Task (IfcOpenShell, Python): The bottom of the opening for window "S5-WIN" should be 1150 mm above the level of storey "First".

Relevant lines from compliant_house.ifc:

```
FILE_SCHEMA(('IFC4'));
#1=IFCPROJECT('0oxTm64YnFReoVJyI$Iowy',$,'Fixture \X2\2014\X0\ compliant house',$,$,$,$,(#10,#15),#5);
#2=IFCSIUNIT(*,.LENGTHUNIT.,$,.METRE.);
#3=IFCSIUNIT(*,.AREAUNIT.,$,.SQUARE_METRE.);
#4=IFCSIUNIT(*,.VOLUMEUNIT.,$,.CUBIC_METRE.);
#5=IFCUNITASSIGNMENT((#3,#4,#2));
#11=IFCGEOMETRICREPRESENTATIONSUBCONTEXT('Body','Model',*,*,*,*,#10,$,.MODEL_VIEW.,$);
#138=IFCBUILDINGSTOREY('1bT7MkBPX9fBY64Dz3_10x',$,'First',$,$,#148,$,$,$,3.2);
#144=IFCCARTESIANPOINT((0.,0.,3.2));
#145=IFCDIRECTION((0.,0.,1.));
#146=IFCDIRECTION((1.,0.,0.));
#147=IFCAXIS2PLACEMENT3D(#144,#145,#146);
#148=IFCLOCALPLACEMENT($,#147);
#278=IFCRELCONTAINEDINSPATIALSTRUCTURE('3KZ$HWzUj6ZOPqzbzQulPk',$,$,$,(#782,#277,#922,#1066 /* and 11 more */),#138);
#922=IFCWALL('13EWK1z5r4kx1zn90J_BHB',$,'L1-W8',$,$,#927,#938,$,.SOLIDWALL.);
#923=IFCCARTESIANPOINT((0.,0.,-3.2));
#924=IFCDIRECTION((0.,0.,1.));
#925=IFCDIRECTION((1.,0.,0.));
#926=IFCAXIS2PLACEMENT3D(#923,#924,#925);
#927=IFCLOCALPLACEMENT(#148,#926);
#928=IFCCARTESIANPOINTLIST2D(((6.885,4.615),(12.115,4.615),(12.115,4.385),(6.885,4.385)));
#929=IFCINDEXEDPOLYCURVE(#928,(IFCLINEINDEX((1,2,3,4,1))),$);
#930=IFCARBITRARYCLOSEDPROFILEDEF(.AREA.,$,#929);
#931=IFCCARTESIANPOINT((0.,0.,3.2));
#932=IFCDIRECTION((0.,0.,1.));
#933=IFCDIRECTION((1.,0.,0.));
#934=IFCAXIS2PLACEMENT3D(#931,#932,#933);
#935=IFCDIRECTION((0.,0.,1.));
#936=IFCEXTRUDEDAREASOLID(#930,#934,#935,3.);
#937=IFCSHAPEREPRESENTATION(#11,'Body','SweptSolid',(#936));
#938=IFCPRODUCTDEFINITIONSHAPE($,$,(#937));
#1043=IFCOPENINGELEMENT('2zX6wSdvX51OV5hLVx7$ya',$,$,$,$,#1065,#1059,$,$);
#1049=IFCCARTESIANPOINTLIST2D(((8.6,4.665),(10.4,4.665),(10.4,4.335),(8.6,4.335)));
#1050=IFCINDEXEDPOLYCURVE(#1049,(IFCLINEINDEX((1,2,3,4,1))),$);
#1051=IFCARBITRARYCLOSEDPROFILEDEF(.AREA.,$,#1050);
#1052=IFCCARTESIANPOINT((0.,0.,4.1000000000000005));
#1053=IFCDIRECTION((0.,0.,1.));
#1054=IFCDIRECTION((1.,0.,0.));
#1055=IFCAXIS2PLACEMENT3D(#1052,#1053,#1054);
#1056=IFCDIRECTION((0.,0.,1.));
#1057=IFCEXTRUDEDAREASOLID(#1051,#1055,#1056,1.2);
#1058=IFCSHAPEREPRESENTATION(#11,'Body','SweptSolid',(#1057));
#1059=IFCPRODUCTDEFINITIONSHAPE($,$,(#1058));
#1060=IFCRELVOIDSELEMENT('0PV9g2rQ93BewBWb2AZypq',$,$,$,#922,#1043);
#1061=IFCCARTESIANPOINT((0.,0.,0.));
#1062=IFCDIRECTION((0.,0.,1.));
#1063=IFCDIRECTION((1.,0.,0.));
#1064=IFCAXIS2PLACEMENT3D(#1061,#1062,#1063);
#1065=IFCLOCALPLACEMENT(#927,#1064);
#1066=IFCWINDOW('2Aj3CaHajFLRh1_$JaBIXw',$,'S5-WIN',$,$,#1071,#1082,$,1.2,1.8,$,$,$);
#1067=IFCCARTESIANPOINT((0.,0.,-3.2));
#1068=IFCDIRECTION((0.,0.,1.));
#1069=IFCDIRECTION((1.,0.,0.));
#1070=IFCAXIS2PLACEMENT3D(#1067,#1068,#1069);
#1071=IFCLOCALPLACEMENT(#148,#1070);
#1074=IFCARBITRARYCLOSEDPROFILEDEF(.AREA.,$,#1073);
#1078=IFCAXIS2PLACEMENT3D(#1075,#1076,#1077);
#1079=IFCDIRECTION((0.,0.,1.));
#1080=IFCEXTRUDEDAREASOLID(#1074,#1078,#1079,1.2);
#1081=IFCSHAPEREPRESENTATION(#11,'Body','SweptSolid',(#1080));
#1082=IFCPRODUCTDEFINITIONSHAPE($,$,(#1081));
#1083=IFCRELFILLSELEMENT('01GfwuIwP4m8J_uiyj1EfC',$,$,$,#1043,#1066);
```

```python
import numpy as np
import ifcopenshell
import ifcopenshell.api.geometry
import ifcopenshell.geom
import ifcopenshell.util.element
import ifcopenshell.util.placement
import ifcopenshell.util.shape
import ifcopenshell.util.unit

model = ifcopenshell.open("compliant_house.ifc")
unit_scale = ifcopenshell.util.unit.calculate_unit_scale(model)

window = model.by_guid("2Aj3CaHajFLRh1_$JaBIXw")
opening = window.FillsVoids[0].RelatingOpeningElement
storey = ifcopenshell.util.element.get_container(window, ifc_class="IfcBuildingStorey")
level = ifcopenshell.util.placement.get_local_placement(storey.ObjectPlacement)[2, 3]

# The opening's origin need not be at the sill, so measure its lowest point.
shape = ifcopenshell.geom.create_shape(ifcopenshell.geom.settings(), opening)
bottom = ifcopenshell.util.shape.get_shape_bottom_elevation(shape, shape.geometry) / unit_scale
dz = level + 1.15 / unit_scale - bottom

shift = np.array([0.0, 0.0, dz])
# The window is not placed relative to its opening, so move both.
for product in (opening, window):
    matrix = ifcopenshell.util.placement.get_local_placement(product.ObjectPlacement)
    matrix[:3, 3] += shift
    ifcopenshell.api.geometry.edit_object_placement(model, product=product, matrix=matrix, is_si=False)

print(f"moved by {dz * unit_scale:+.3f} m")

model.write("compliant_house_edited.ifc")
```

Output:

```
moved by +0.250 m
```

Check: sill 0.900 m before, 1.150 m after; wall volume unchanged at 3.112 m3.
